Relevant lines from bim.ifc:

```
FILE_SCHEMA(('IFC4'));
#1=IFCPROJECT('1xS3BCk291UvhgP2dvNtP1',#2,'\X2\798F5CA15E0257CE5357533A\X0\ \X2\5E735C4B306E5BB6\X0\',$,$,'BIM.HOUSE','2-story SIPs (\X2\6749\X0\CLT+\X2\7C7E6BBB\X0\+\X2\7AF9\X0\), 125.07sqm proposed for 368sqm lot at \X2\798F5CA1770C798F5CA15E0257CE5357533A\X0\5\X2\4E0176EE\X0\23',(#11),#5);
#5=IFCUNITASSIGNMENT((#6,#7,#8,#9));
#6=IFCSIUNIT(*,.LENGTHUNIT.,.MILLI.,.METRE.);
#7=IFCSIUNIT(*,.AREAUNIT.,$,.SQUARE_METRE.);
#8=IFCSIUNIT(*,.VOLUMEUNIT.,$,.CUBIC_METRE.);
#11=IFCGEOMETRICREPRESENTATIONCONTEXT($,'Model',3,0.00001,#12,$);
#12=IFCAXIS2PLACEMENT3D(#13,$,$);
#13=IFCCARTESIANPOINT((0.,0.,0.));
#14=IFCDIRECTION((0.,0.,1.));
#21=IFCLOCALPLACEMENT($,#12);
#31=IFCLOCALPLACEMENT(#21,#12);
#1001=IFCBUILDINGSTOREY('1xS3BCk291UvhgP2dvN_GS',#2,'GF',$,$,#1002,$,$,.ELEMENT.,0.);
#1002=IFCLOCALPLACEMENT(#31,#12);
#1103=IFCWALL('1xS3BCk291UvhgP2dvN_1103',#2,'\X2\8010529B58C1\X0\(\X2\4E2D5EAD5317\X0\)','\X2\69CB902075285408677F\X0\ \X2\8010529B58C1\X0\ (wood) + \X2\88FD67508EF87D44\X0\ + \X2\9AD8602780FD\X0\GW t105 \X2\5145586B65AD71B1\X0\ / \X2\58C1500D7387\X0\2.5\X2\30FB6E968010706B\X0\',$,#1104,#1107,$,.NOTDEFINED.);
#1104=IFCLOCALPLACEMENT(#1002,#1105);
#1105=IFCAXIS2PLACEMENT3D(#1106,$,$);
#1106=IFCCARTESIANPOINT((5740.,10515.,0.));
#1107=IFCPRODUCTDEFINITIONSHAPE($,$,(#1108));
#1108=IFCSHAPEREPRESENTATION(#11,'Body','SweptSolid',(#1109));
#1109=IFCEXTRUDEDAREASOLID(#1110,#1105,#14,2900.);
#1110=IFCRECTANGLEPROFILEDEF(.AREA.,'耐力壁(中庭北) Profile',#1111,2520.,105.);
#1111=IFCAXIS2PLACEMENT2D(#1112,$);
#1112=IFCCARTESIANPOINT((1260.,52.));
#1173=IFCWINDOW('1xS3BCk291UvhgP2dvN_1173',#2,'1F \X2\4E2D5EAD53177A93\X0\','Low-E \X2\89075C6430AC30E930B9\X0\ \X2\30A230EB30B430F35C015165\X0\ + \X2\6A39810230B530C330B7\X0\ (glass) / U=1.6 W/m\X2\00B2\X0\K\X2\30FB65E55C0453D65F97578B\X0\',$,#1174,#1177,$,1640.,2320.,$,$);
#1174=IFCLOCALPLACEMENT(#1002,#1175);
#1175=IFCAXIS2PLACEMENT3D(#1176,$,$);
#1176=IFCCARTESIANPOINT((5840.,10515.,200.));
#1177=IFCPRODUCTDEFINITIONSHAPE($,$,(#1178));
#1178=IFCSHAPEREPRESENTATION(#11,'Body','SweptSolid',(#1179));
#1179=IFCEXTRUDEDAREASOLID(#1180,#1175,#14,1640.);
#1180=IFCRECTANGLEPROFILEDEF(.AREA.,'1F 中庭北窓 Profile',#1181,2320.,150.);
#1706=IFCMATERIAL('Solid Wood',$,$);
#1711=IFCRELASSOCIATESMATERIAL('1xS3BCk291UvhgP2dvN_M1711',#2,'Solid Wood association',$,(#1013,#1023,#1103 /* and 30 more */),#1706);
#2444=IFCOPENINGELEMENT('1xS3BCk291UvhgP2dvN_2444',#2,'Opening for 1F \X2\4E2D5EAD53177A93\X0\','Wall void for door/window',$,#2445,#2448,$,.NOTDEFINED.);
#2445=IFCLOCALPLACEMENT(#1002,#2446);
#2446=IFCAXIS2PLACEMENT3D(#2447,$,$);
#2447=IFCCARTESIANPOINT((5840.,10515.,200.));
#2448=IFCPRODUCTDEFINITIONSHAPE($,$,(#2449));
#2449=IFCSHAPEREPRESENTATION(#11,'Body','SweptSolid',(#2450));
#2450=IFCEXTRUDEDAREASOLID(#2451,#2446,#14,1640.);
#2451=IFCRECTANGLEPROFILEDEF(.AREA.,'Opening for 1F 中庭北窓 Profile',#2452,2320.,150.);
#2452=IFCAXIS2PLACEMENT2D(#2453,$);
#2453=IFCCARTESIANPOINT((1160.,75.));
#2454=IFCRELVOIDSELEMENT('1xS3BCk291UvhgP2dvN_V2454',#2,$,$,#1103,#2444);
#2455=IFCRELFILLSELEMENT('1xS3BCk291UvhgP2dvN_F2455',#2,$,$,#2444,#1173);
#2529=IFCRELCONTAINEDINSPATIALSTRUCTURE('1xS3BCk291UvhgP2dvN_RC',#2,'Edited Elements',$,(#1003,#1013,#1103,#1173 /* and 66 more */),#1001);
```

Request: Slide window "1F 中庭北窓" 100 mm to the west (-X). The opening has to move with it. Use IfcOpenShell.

```python
import ifcopenshell
import ifcopenshell.api.geometry
import ifcopenshell.util.placement
import ifcopenshell.util.unit

model = ifcopenshell.open("bim.ifc")
unit_scale = ifcopenshell.util.unit.calculate_unit_scale(model)

window = model.by_guid("1xS3BCk291UvhgP2dvN_1173")
opening = window.FillsVoids[0].RelatingOpeningElement
wall = opening.VoidsElements[0].RelatingBuildingElement

wall_matrix = ifcopenshell.util.placement.get_local_placement(wall.ObjectPlacement)
shift = wall_matrix[:3, 0] * -0.1 / unit_scale
before = ifcopenshell.util.placement.get_local_placement(window.ObjectPlacement)[:3, 3].copy()

# The window is not placed relative to its opening, so move both.
for product in (opening, window):
    matrix = ifcopenshell.util.placement.get_local_placement(product.ObjectPlacement)
    matrix[:3, 3] += shift
    ifcopenshell.api.geometry.edit_object_placement(model, product=product, matrix=matrix, is_si=False)

after = ifcopenshell.util.placement.get_local_placement(window.ObjectPlacement)[:3, 3]
print("window moved by", (after - before).round(3) + 0.0)

model.write("bim_rev.ifc")
```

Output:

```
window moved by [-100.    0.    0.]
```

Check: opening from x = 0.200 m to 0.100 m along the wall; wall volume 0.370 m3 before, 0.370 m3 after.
